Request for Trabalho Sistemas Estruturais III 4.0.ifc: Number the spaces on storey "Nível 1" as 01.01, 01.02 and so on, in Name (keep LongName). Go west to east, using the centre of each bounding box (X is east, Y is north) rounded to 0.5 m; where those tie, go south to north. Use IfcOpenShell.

First a look at what the model holds.

```python
import ifcopenshell
import ifcopenshell.util.element
import ifcopenshell.util.placement

model = ifcopenshell.open("Trabalho Sistemas Estruturais III 4.0.ifc")
print(model.schema)
storey = next(s for s in model.by_type("IfcBuildingStorey") if s.Name == "Nível 1")
spaces = [e for e in ifcopenshell.util.element.get_decomposition(storey) if e.is_a("IfcSpace")]
for e in sorted(spaces, key=lambda e: e.id()):
    origin = ifcopenshell.util.placement.get_local_placement(e.ObjectPlacement)[:3, 3]
    print(e.id(), e.Name, e.LongName, origin.round(2) + 0.0, sep=" | ")
```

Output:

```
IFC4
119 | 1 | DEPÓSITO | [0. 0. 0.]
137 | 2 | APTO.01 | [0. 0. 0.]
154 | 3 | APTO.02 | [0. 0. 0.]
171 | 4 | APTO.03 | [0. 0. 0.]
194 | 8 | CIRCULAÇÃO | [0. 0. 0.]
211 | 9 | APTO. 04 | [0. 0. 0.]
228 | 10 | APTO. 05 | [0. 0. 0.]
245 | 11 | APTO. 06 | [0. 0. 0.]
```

```python
import ifcopenshell
import ifcopenshell.geom
import ifcopenshell.util.element
import ifcopenshell.util.shape

model = ifcopenshell.open("Trabalho Sistemas Estruturais III 4.0.ifc")
settings = ifcopenshell.geom.settings()
settings.set("use-world-coords", True)


def centre(element):
    shape = ifcopenshell.geom.create_shape(settings, element)
    return ifcopenshell.util.shape.get_bbox_centroid(shape.geometry)


storey = next(s for s in model.by_type("IfcBuildingStorey") if s.Name == "Nível 1")
spaces = [e for e in ifcopenshell.util.element.get_decomposition(storey) if e.is_a("IfcSpace")]

# Insertion points can sit at a corner or the storey origin, so sort by the geometry (in metres).
centres = {e: centre(e) for e in spaces}
spaces.sort(key=lambda e: (round(centres[e][0] / 0.5), centres[e][1]))

for i, e in enumerate(spaces, start=1):
    number = f"01.{i:02d}"
    e.Name = number
    print(e.id(), number)

model.write("Trabalho Sistemas Estruturais III 4.0_edited.ifc")
```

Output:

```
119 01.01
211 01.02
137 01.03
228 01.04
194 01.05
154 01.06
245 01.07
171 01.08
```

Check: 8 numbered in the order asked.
